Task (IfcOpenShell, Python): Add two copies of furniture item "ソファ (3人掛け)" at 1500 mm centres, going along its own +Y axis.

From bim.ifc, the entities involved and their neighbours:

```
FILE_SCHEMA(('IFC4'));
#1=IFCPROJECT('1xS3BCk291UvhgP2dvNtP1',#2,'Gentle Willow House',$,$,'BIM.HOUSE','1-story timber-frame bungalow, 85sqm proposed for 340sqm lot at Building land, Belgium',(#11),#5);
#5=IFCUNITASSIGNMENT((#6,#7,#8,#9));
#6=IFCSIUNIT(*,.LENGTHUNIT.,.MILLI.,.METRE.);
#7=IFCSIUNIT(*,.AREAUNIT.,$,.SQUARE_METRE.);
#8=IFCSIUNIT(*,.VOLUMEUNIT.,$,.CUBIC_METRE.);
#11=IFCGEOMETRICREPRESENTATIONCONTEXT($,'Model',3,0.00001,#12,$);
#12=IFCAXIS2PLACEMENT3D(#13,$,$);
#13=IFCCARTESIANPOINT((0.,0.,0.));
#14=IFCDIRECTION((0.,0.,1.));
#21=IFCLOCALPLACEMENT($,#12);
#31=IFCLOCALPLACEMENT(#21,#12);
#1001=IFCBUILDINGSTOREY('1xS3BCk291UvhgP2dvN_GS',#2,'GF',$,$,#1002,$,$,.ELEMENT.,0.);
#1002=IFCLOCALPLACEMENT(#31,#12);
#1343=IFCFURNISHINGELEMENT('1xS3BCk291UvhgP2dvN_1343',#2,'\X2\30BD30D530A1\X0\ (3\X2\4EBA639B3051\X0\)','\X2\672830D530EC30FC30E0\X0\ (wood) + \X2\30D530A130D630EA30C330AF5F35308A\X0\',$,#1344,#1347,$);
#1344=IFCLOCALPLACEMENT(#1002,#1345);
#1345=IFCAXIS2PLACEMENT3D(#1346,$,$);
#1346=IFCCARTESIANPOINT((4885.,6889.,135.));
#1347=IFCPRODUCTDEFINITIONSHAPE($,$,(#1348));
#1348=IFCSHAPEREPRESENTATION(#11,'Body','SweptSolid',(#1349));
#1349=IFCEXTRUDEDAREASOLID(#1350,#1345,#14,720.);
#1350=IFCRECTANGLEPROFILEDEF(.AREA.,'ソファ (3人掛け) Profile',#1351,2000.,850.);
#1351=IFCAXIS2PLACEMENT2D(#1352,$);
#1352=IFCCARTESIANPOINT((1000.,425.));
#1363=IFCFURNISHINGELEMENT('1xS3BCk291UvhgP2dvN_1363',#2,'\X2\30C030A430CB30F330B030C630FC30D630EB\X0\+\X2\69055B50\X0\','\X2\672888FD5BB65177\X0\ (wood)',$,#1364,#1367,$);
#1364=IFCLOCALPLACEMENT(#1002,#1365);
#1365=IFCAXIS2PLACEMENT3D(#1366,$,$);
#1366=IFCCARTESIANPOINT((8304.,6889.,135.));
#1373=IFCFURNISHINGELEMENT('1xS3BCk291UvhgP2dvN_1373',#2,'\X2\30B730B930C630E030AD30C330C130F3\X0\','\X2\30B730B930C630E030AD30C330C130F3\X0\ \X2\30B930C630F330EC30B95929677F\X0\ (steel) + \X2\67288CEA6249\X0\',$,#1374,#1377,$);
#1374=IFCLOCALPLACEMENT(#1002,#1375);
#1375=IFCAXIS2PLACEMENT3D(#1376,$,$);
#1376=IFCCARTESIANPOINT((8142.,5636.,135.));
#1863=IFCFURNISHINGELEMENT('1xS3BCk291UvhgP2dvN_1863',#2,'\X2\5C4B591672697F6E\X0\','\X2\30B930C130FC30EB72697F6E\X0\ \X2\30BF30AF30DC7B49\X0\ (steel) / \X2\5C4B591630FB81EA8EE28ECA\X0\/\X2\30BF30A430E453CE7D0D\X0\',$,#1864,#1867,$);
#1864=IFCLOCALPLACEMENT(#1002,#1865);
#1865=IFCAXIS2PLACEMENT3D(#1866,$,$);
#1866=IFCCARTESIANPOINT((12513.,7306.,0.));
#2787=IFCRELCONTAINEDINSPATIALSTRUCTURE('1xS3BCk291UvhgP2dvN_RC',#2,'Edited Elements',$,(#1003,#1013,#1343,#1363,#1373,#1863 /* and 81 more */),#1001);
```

```python
import ifcopenshell
import ifcopenshell.api.geometry
import ifcopenshell.api.root
import ifcopenshell.util.element
import ifcopenshell.util.placement
import ifcopenshell.util.unit

model = ifcopenshell.open("bim.ifc")
unit_scale = ifcopenshell.util.unit.calculate_unit_scale(model)


def reuse_history(source, copy):
    """copy_class also copies each property set's owner history, people and application; keep the originals."""
    for rel in copy.IsDefinedBy:
        if rel.is_a("IfcRelDefinesByProperties") and (history := rel.RelatingPropertyDefinition.OwnerHistory):
            rel.RelatingPropertyDefinition.OwnerHistory = source.OwnerHistory
            ifcopenshell.util.element.remove_deep2(model, history)


source = model.by_id(1343)
base = ifcopenshell.util.placement.get_local_placement(source.ObjectPlacement)
step = base[:3, 1] * 1.5 / unit_scale

for i in range(1, 3):
    copy = ifcopenshell.api.root.copy_class(model, product=source)
    copy.Representation = ifcopenshell.util.element.copy_deep(
        model, source.Representation, exclude=["IfcGeometricRepresentationContext", "IfcRepresentationMap"]
    )
    reuse_history(source, copy)
    matrix = base.copy()
    matrix[:3, 3] += i * step
    print("added at", matrix[:3, 3].round(3) + 0.0)
    ifcopenshell.api.geometry.edit_object_placement(model, product=copy, matrix=matrix, is_si=False)

model.write("bim-out.ifc")
```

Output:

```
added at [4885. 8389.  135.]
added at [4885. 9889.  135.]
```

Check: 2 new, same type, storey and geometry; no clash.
